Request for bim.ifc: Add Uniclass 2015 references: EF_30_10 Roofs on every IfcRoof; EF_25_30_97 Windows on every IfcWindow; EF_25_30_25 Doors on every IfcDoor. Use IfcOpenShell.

First a look at what the model holds.

```python
import ifcopenshell

model = ifcopenshell.open("bim.ifc")
print(model.schema)
print("classifications:", [c.Name for c in model.by_type("IfcClassification")])
for ifc_class in ("IfcDoor", "IfcRoof", "IfcStair", "IfcWall", "IfcWindow"):
    print(ifc_class, len(model.by_type(ifc_class)))
```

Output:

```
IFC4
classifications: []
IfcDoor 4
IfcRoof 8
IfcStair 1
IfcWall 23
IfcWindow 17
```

```python
import ifcopenshell
import ifcopenshell.api.classification

model = ifcopenshell.open("bim.ifc")

system = ifcopenshell.api.classification.add_classification(model, classification="Uniclass 2015")

codes = {
    "IfcRoof": ("EF_30_10", "Roofs"),
    "IfcWindow": ("EF_25_30_97", "Windows"),
    "IfcDoor": ("EF_25_30_25", "Doors"),
}
for ifc_class, (code, name) in codes.items():
    products = model.by_type(ifc_class)
    ifcopenshell.api.classification.add_reference(
        model, products=products, classification=system, identification=code, name=name
    )
    print(code, len(products))

model.write("bim_updated.ifc")
```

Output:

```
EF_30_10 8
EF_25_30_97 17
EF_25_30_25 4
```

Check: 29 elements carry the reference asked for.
